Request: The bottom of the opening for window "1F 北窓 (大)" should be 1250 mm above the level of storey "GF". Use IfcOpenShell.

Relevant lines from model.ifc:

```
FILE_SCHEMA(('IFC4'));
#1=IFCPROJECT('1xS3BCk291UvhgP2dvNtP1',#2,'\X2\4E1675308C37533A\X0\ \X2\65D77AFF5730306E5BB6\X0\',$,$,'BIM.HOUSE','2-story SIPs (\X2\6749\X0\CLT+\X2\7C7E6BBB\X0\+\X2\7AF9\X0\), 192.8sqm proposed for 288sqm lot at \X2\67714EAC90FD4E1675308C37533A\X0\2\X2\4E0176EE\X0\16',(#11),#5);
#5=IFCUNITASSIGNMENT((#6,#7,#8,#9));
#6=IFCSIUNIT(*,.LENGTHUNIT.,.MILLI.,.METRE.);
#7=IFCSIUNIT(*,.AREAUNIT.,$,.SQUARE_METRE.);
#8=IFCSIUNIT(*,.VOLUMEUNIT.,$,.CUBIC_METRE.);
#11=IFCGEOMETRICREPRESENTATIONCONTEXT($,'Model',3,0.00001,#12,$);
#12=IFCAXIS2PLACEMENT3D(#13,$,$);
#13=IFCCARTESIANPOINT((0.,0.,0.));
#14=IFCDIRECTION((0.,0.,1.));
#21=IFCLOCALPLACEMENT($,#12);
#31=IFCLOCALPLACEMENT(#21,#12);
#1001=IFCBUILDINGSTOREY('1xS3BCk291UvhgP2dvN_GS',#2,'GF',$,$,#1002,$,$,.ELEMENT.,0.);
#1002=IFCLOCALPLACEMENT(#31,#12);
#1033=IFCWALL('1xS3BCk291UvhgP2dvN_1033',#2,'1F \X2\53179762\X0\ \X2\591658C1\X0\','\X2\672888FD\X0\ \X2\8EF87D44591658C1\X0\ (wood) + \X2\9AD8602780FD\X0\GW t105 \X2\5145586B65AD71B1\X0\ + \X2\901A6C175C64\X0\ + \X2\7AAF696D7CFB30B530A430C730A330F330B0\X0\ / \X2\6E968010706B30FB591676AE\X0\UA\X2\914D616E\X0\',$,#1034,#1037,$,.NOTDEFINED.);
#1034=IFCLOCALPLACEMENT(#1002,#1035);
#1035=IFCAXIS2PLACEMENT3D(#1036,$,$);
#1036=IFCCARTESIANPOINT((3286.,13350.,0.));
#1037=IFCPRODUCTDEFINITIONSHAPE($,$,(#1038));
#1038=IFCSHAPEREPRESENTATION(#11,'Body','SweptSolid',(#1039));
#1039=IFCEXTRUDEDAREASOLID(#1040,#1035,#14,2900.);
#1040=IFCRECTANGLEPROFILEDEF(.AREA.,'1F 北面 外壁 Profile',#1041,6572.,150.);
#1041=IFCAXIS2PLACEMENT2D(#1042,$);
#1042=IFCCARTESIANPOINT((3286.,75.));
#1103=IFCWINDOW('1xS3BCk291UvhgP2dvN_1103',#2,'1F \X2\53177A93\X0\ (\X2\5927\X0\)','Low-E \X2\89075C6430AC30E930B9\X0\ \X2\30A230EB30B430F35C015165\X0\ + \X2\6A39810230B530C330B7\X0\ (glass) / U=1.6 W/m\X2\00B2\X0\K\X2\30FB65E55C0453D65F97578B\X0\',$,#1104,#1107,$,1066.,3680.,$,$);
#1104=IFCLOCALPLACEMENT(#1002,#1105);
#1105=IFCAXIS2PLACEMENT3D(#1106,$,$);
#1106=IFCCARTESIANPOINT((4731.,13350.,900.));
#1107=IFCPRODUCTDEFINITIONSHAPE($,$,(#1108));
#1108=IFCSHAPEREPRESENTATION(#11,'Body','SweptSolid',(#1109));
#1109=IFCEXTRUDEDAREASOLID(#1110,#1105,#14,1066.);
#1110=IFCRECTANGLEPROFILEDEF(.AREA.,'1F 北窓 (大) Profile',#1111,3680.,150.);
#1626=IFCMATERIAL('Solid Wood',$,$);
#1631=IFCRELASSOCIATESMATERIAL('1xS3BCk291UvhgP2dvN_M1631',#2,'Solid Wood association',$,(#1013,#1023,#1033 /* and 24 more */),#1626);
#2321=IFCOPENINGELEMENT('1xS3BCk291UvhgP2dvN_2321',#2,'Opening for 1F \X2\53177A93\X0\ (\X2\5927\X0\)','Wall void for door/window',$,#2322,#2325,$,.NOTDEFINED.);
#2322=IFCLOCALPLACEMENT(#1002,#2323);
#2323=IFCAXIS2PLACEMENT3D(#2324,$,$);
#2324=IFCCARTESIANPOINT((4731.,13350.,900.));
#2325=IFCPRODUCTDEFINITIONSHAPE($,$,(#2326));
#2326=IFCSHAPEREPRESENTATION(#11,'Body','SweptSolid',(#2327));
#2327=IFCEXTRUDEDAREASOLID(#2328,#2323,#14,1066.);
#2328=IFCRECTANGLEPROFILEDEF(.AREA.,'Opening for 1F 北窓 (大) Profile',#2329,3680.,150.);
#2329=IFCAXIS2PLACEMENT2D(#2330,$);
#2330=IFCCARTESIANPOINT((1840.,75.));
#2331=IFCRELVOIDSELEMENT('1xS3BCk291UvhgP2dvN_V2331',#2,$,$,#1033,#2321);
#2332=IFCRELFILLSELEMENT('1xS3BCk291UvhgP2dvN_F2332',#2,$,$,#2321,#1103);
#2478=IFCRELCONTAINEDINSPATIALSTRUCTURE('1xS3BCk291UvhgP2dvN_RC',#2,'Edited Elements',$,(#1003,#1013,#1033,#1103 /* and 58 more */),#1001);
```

```python
import numpy as np
import ifcopenshell
import ifcopenshell.api.geometry
import ifcopenshell.geom
import ifcopenshell.util.element
import ifcopenshell.util.placement
import ifcopenshell.util.shape
import ifcopenshell.util.unit

model = ifcopenshell.open("model.ifc")
unit_scale = ifcopenshell.util.unit.calculate_unit_scale(model)

window = model.by_id(1103)
opening = window.FillsVoids[0].RelatingOpeningElement
storey = ifcopenshell.util.element.get_container(window, ifc_class="IfcBuildingStorey")
level = ifcopenshell.util.placement.get_local_placement(storey.ObjectPlacement)[2, 3]

# The opening's origin need not be at the sill, so measure its lowest point.
shape = ifcopenshell.geom.create_shape(ifcopenshell.geom.settings(), opening)
bottom = ifcopenshell.util.shape.get_shape_bottom_elevation(shape, shape.geometry) / unit_scale
dz = level + 1.25 / unit_scale - bottom

shift = np.array([0.0, 0.0, dz])
# The window is not placed relative to its opening, so move both.
for product in (opening, window):
    matrix = ifcopenshell.util.placement.get_local_placement(product.ObjectPlacement)
    matrix[:3, 3] += shift
    ifcopenshell.api.geometry.edit_object_placement(model, product=product, matrix=matrix, is_si=False)

print(f"moved by {dz * unit_scale:+.3f} m")

model.write("model_updated.ifc")
```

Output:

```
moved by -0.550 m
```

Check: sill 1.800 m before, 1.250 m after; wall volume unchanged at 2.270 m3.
